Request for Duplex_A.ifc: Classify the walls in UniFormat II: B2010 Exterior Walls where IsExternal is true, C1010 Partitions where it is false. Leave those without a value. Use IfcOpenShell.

First a look at what the model holds.

```python
import ifcopenshell
import ifcopenshell.util.element

model = ifcopenshell.open("Duplex_A.ifc")
print(model.schema)
print("classifications:", [c.Name for c in model.by_type("IfcClassification")])
values = [ifcopenshell.util.element.get_pset(e, "Pset_WallCommon", "IsExternal") for e in model.by_type("IfcWall")]
for value in (True, False, None):
    print("IsExternal", value, values.count(value))
```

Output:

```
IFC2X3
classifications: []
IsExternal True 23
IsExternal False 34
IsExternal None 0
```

```python
import ifcopenshell
import ifcopenshell.api.classification
import ifcopenshell.util.element

model = ifcopenshell.open("Duplex_A.ifc")

# IFC2X3 requires Source and Edition and has no link from the project to the system.
system = model.create_entity("IfcClassification", Source="ASTM", Edition="E1557", Name="UniFormat II")

walls = model.by_type("IfcWall")
external = {e: ifcopenshell.util.element.get_pset(e, "Pset_WallCommon", "IsExternal") for e in walls}
for flag, code, name in ((True, "B2010", "Exterior Walls"), (False, "C1010", "Partitions")):
    products = [e for e in walls if external[e] is flag]
    ifcopenshell.api.classification.add_reference(
        model, products=products, classification=system, identification=code, name=name
    )
    print(code, len(products))

model.write("Duplex_A_edited.ifc")
```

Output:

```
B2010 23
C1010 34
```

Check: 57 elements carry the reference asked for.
